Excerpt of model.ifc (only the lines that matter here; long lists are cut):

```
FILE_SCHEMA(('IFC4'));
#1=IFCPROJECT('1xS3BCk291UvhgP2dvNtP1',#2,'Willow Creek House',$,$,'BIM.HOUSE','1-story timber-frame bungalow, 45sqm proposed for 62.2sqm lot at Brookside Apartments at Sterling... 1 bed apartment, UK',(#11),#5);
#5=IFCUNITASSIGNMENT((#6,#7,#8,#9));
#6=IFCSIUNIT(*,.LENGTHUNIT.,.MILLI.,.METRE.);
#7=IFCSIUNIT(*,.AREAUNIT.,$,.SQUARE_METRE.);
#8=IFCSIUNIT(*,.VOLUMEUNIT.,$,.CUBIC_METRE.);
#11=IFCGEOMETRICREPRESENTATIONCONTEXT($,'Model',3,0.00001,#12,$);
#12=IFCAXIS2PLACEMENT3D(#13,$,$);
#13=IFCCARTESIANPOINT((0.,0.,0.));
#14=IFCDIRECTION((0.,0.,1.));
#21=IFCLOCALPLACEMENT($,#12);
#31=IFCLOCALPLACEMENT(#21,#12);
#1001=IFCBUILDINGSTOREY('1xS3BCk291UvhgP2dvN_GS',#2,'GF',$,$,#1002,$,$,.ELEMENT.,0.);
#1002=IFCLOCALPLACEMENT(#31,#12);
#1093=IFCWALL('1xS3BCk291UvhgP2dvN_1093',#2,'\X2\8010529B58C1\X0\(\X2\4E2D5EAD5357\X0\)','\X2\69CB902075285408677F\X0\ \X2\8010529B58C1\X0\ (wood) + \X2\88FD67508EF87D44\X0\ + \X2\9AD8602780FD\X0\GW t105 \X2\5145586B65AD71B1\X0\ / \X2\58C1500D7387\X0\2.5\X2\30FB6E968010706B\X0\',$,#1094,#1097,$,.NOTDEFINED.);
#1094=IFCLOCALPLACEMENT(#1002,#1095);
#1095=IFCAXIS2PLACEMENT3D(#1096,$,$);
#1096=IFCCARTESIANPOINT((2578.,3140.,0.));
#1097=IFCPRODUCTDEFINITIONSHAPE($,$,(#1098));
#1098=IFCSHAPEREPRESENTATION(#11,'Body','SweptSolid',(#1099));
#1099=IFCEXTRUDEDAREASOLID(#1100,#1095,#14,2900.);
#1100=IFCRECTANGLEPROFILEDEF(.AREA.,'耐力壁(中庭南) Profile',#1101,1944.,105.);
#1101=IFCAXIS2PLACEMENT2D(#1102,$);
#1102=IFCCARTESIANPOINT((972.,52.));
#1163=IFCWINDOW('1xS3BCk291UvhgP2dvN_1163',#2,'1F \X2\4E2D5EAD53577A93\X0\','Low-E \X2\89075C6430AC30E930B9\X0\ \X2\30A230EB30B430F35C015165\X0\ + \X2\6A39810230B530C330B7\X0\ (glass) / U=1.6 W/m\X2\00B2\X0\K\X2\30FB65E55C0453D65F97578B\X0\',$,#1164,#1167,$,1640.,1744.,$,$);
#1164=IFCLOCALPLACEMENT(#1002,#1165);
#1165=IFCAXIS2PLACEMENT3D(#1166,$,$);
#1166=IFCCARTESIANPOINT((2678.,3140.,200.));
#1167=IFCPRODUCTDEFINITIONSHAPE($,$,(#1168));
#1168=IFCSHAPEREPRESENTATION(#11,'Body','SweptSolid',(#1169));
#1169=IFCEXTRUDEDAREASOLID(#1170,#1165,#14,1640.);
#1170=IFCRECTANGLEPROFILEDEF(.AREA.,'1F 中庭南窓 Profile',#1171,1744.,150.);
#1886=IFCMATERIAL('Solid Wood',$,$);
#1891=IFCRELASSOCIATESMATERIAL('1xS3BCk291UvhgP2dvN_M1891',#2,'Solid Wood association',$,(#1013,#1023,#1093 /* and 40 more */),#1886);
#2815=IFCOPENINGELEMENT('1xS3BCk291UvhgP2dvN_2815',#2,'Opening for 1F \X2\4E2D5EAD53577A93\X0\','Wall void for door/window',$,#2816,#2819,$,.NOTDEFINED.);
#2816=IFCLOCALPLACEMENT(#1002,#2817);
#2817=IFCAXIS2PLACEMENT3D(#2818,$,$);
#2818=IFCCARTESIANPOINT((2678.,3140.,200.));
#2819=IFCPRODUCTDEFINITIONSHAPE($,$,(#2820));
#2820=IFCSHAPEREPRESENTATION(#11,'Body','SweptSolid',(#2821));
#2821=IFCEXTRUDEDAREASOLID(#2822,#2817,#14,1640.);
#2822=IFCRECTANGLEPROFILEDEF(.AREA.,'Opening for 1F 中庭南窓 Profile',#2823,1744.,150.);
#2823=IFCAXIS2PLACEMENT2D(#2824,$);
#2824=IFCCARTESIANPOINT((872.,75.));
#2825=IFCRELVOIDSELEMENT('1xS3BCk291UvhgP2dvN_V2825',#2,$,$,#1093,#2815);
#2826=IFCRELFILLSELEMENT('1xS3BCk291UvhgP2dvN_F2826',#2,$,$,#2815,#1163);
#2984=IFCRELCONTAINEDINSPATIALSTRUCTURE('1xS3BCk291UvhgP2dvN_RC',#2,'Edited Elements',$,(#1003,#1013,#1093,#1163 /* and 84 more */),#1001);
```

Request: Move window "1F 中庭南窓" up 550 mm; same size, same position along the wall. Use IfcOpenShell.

```python
import numpy as np
import ifcopenshell
import ifcopenshell.api.geometry
import ifcopenshell.util.placement
import ifcopenshell.util.unit

model = ifcopenshell.open("model.ifc")
unit_scale = ifcopenshell.util.unit.calculate_unit_scale(model)

window = model.by_guid("1xS3BCk291UvhgP2dvN_1163")
opening = window.FillsVoids[0].RelatingOpeningElement
dz = 0.55 / unit_scale

shift = np.array([0.0, 0.0, dz])
# The window is not placed relative to its opening, so move both.
for product in (opening, window):
    matrix = ifcopenshell.util.placement.get_local_placement(product.ObjectPlacement)
    matrix[:3, 3] += shift
    ifcopenshell.api.geometry.edit_object_placement(model, product=product, matrix=matrix, is_si=False)

print(f"moved by {dz * unit_scale:+.3f} m")

model.write("model_updated.ifc")
```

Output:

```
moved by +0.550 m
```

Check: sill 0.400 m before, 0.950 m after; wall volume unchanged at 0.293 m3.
